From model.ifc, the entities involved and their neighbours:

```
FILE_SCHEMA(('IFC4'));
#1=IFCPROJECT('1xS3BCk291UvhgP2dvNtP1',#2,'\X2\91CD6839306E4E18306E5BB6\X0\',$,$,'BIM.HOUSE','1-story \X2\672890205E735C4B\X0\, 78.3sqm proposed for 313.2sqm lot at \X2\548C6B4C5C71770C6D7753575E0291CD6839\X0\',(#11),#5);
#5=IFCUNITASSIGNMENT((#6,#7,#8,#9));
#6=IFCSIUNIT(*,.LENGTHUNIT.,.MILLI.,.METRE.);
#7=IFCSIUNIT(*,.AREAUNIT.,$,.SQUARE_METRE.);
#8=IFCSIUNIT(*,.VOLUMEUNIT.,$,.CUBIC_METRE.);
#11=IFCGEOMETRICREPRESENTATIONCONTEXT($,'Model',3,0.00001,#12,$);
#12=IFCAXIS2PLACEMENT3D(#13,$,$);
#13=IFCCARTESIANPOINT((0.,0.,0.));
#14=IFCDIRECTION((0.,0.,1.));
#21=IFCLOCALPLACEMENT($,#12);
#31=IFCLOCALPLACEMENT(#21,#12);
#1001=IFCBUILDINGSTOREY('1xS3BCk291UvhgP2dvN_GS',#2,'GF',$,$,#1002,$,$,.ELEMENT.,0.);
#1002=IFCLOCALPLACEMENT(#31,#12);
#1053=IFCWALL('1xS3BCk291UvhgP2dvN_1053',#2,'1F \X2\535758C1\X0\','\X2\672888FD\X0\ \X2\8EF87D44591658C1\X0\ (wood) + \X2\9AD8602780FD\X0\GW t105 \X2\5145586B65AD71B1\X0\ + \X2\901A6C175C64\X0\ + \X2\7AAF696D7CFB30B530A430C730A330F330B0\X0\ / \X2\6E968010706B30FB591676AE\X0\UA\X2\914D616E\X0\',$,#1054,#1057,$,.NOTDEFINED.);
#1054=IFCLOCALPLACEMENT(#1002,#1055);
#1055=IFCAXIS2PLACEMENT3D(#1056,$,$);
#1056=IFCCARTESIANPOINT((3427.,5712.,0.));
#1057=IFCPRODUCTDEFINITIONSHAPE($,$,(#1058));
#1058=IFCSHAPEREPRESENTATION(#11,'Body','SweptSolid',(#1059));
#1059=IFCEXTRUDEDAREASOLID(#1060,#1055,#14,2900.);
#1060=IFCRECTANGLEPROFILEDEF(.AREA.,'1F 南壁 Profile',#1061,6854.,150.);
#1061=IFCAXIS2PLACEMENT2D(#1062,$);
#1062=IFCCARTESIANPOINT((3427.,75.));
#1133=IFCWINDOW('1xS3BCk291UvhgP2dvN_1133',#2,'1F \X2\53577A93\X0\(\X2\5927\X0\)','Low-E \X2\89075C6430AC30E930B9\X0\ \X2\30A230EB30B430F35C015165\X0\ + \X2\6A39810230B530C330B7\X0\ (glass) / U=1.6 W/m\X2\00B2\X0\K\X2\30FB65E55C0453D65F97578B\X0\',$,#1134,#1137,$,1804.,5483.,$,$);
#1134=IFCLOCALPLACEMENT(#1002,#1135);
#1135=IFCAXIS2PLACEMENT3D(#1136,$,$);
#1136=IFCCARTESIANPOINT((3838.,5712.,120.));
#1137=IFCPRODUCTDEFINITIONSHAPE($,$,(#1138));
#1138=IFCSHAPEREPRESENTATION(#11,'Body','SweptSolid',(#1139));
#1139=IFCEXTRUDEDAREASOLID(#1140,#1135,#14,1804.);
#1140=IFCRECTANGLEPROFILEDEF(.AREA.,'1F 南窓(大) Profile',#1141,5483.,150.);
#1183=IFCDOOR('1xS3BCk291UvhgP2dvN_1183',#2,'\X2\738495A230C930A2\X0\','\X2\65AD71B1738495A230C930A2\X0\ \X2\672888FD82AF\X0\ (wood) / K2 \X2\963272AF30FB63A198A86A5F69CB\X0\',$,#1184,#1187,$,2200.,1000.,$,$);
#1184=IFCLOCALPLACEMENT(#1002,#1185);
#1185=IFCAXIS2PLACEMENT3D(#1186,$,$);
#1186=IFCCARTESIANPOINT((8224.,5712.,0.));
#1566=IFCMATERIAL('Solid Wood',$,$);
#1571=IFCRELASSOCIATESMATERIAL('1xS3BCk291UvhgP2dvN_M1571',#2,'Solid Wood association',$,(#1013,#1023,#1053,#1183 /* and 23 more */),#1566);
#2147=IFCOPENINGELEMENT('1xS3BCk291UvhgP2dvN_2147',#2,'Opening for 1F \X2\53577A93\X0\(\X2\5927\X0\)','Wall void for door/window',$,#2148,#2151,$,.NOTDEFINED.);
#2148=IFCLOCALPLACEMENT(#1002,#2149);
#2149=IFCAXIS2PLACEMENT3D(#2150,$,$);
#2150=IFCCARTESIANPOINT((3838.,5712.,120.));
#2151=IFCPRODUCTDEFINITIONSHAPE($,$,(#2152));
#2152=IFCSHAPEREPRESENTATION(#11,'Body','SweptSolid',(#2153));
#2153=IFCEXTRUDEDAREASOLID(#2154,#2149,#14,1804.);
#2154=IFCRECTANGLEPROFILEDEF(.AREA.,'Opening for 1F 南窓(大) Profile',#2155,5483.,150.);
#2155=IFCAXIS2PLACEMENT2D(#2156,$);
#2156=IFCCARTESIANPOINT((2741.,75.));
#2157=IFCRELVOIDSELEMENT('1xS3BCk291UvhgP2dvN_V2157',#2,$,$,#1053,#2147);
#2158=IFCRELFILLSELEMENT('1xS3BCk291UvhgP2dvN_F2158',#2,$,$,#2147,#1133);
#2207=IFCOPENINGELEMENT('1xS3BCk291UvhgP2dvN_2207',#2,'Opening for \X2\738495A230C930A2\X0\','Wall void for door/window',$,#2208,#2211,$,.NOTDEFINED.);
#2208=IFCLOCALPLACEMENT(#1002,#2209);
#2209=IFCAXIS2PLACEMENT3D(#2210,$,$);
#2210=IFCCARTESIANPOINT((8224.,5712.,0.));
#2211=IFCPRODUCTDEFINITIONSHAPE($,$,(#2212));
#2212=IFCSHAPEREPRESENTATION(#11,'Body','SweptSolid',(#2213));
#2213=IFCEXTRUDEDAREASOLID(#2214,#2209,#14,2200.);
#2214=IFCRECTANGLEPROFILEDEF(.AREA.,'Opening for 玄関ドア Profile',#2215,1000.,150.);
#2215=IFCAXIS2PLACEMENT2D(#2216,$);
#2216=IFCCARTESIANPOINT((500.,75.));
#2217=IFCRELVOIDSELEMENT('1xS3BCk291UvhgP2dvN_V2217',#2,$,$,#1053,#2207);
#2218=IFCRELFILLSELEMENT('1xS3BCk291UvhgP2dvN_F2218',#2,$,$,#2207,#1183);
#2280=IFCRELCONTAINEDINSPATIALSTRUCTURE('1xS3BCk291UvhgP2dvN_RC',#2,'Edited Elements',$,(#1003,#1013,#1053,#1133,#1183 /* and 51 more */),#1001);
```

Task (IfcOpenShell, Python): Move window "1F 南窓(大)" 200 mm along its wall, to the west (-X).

```python
import ifcopenshell
import ifcopenshell.api.geometry
import ifcopenshell.util.placement
import ifcopenshell.util.unit

model = ifcopenshell.open("model.ifc")
unit_scale = ifcopenshell.util.unit.calculate_unit_scale(model)

window = model.by_guid("1xS3BCk291UvhgP2dvN_1133")
opening = window.FillsVoids[0].RelatingOpeningElement
wall = opening.VoidsElements[0].RelatingBuildingElement

wall_matrix = ifcopenshell.util.placement.get_local_placement(wall.ObjectPlacement)
shift = wall_matrix[:3, 0] * -0.2 / unit_scale
before = ifcopenshell.util.placement.get_local_placement(window.ObjectPlacement)[:3, 3].copy()

# The window is not placed relative to its opening, so move both.
for product in (opening, window):
    matrix = ifcopenshell.util.placement.get_local_placement(product.ObjectPlacement)
    matrix[:3, 3] += shift
    ifcopenshell.api.geometry.edit_object_placement(model, product=product, matrix=matrix, is_si=False)

after = ifcopenshell.util.placement.get_local_placement(window.ObjectPlacement)[:3, 3]
print("window moved by", (after - before).round(3) + 0.0)

model.write("model_edited.ifc")
```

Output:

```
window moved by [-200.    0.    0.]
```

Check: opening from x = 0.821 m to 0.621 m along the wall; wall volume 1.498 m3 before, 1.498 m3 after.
